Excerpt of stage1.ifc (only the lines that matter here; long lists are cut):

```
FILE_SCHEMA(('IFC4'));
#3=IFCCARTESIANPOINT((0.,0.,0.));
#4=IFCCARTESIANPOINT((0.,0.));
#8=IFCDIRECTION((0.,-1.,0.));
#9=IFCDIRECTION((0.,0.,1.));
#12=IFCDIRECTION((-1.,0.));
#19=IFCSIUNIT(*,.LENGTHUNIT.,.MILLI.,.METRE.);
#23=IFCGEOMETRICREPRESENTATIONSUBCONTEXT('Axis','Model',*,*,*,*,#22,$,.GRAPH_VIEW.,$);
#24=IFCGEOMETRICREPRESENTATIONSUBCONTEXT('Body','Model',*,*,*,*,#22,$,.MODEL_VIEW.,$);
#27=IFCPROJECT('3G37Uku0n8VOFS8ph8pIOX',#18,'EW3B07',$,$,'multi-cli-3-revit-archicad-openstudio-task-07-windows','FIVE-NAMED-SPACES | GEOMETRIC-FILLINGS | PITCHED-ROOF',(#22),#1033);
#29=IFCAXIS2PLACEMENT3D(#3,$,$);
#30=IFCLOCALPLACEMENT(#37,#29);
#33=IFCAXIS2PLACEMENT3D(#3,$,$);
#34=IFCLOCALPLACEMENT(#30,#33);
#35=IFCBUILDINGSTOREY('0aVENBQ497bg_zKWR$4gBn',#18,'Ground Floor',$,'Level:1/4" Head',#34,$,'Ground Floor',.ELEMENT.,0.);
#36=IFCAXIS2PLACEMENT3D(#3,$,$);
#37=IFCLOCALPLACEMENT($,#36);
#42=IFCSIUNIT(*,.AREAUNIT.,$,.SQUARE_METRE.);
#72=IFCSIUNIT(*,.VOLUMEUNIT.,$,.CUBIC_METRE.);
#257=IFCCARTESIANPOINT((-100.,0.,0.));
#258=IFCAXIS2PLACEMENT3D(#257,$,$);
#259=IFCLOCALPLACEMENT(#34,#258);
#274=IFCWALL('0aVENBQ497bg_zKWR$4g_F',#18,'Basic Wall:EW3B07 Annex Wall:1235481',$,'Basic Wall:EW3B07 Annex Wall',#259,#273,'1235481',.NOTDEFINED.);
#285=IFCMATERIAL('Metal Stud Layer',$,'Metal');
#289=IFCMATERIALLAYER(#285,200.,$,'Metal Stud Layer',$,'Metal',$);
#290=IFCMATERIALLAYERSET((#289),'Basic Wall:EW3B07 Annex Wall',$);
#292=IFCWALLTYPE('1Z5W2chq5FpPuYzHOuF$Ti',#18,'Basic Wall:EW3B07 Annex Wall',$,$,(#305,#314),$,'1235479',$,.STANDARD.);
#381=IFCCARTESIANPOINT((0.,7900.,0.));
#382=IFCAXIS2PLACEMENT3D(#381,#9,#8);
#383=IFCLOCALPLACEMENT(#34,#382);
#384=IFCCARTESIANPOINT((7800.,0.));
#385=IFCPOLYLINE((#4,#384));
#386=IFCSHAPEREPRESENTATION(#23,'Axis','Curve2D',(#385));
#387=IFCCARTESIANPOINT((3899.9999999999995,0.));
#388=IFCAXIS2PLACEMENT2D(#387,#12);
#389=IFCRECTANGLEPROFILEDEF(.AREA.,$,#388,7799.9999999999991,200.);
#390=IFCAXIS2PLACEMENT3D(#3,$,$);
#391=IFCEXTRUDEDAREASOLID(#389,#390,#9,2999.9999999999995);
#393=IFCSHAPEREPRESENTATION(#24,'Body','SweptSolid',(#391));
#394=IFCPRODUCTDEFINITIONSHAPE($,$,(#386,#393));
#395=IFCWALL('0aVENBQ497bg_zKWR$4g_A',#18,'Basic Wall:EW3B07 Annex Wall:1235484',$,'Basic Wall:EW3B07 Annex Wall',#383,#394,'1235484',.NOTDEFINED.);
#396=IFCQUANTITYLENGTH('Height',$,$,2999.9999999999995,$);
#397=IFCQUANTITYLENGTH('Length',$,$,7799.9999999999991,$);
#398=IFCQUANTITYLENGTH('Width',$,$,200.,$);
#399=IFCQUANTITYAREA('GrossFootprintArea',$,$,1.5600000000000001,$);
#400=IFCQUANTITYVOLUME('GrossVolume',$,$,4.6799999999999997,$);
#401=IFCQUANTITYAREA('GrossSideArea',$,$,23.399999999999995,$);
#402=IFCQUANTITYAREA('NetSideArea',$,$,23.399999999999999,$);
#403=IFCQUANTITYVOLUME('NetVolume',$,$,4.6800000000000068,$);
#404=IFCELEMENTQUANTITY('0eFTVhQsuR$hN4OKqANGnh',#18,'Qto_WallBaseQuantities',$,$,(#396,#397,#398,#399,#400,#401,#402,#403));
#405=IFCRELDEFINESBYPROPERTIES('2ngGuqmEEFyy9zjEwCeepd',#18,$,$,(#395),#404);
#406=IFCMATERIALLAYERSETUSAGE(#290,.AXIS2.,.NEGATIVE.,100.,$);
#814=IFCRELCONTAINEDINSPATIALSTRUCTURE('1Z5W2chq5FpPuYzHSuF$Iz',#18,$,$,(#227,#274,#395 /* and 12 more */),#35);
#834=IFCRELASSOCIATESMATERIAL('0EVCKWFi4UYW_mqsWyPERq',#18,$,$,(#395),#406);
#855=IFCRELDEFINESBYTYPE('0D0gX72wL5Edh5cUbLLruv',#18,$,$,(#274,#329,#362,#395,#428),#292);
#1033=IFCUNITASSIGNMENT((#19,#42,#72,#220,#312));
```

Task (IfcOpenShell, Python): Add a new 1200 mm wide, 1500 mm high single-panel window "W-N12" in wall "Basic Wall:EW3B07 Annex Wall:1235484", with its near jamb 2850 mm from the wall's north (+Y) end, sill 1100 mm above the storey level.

```python
import numpy as np
import ifcopenshell
import ifcopenshell.api.feature
import ifcopenshell.api.geometry
import ifcopenshell.api.pset
import ifcopenshell.api.root
import ifcopenshell.api.spatial
import ifcopenshell.geom
import ifcopenshell.util.element
import ifcopenshell.util.placement
import ifcopenshell.util.representation
import ifcopenshell.util.shape
import ifcopenshell.util.unit

model = ifcopenshell.open("stage1.ifc")
unit_scale = ifcopenshell.util.unit.calculate_unit_scale(model)
area_scale = ifcopenshell.util.unit.calculate_unit_scale(model, "AREAUNIT")
volume_scale = ifcopenshell.util.unit.calculate_unit_scale(model, "VOLUMEUNIT")
settings = ifcopenshell.geom.settings()


def volume(element):
    """Net volume in cubic metres, openings subtracted."""
    shape = ifcopenshell.geom.create_shape(settings, element)
    return ifcopenshell.util.shape.get_volume(shape.geometry)


wall = model.by_guid("0aVENBQ497bg_zKWR$4g_A")
storey = ifcopenshell.util.element.get_container(wall, ifc_class="IfcBuildingStorey")
context = ifcopenshell.util.representation.get_context(model, "Model", "Body", "MODEL_VIEW")
before = volume(wall)

width, height, from_end, sill = 1.2, 1.5, 2.85, 1.1  # metres

# The wall runs along its own X axis, and the end named is its -X end.
wall_shape = ifcopenshell.geom.create_shape(settings, wall)
x, y, z = ifcopenshell.util.shape.get_vertices(wall_shape.geometry).T
start = x.min() + from_end
face, thickness = float(y.min()), float(y.max() - y.min())
wall_matrix = ifcopenshell.util.placement.get_local_placement(wall.ObjectPlacement)
level = ifcopenshell.util.placement.get_local_placement(storey.ObjectPlacement)[2, 3]


def in_wall(x, y):
    """Placement at x, y metres in the wall's axes, at sill height."""
    matrix = wall_matrix.copy()
    matrix[:, 3] = wall_matrix @ np.array([x / unit_scale, y / unit_scale, 0.0, 1.0])
    matrix[2, 3] = level + sill / unit_scale
    return matrix


# Opening: a box that overshoots both wall faces by 50 mm.
opening = ifcopenshell.api.root.create_entity(model, ifc_class="IfcOpeningElement", predefined_type="OPENING")
box = ifcopenshell.api.geometry.add_wall_representation(
    model, context=context, length=width, height=height, thickness=thickness + 0.1
)
ifcopenshell.api.geometry.assign_representation(model, product=opening, representation=box)
ifcopenshell.api.geometry.edit_object_placement(model, product=opening, matrix=in_wall(start, face - 0.05), is_si=False)
ifcopenshell.api.feature.add_feature(model, feature=opening, element=wall)

window = ifcopenshell.api.root.create_entity(model, ifc_class="IfcWindow", name="W-N12", predefined_type="WINDOW")
window.OverallWidth, window.OverallHeight = width / unit_scale, height / unit_scale
window.PartitioningType = "SINGLE_PANEL"
body = ifcopenshell.api.geometry.add_window_representation(
    model,
    context=context,
    overall_width=window.OverallWidth,
    overall_height=window.OverallHeight,
    partition_type="SINGLE_PANEL",
)
ifcopenshell.api.geometry.assign_representation(model, product=window, representation=body)
ifcopenshell.api.spatial.assign_container(model, products=[window], relating_structure=storey)
ifcopenshell.api.feature.add_filling(model, opening=opening, element=window)

# Centre the window in the wall's thickness.
ifcopenshell.api.geometry.edit_object_placement(model, product=window, matrix=in_wall(start, face), is_si=False)
window_shape = ifcopenshell.geom.create_shape(settings, window)
depth = ifcopenshell.util.shape.get_vertices(window_shape.geometry)[:, 1]
offset = face + thickness / 2 - (depth.min() + depth.max()) / 2
ifcopenshell.api.geometry.edit_object_placement(model, product=window, matrix=in_wall(start, offset), is_si=False)

after = volume(wall)

# Update the wall's stored quantities.
qto = model.by_id(ifcopenshell.util.element.get_pset(wall, "Qto_WallBaseQuantities", should_inherit=False)["id"])
ifcopenshell.api.pset.edit_qto(model, qto=qto, properties={
    "NetSideArea": after / thickness / area_scale,
    "NetVolume": after / volume_scale,
})

print(f"wall volume {before:.3f} -> {after:.3f} m3")

model.write("stage1_updated.ifc")
```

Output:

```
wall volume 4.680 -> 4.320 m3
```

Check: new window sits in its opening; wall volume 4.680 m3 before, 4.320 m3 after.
